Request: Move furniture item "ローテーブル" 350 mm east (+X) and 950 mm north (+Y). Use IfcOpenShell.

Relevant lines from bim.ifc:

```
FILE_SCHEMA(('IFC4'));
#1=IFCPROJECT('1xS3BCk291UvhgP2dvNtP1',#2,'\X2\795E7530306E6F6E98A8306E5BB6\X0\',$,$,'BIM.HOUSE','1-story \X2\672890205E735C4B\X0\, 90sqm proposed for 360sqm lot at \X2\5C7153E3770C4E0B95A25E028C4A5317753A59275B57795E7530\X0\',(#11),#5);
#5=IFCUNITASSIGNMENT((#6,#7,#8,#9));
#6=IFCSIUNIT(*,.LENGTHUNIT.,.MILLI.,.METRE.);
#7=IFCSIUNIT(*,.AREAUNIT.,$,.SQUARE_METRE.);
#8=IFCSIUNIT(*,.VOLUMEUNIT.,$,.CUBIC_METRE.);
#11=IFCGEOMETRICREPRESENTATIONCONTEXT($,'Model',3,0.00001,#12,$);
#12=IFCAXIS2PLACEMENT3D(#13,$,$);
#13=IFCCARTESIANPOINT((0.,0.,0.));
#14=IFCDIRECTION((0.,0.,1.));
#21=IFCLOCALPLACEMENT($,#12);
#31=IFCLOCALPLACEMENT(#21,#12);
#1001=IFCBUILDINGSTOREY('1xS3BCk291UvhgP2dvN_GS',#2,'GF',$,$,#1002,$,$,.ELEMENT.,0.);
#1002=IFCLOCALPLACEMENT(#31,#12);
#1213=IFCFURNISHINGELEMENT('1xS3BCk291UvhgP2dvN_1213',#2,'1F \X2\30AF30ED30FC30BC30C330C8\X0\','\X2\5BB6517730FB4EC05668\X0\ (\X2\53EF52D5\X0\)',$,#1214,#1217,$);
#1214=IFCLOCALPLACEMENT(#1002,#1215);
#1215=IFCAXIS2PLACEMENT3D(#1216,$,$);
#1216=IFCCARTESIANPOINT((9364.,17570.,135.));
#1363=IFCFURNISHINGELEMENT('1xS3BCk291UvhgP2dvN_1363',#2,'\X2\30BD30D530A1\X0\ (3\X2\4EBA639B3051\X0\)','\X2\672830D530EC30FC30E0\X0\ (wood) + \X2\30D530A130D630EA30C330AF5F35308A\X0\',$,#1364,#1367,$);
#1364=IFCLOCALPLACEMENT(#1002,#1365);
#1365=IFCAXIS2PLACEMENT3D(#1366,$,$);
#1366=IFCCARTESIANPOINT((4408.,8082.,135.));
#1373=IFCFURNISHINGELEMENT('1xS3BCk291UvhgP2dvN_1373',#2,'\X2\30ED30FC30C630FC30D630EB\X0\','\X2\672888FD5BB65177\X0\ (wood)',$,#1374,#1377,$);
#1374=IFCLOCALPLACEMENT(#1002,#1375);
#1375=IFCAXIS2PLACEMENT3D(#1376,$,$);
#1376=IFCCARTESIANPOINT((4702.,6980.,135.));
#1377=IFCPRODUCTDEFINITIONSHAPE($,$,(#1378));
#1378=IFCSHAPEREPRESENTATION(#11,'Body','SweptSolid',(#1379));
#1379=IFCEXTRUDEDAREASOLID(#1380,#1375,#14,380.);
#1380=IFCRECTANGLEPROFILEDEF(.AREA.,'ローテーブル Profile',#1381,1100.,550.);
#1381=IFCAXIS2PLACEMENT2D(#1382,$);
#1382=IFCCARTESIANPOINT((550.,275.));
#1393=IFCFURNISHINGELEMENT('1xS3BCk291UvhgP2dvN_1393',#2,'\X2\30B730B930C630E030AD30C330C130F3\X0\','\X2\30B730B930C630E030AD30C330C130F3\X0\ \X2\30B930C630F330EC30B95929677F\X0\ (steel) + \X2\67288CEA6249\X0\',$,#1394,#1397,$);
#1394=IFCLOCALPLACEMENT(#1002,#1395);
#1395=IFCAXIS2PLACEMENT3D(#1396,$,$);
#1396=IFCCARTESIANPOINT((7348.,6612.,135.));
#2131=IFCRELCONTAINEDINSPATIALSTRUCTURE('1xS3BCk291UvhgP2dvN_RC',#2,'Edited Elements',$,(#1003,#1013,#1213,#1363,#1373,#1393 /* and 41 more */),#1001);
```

```python
import ifcopenshell
import ifcopenshell.api.geometry
import ifcopenshell.util.placement
import ifcopenshell.util.unit

model = ifcopenshell.open("bim.ifc")
unit_scale = ifcopenshell.util.unit.calculate_unit_scale(model)

item = model.by_guid("1xS3BCk291UvhgP2dvN_1373")
matrix = ifcopenshell.util.placement.get_local_placement(item.ObjectPlacement)
matrix[0, 3] += 0.35 / unit_scale
matrix[1, 3] += 0.95 / unit_scale
ifcopenshell.api.geometry.edit_object_placement(model, product=item, matrix=matrix, is_si=False)

print(ifcopenshell.util.placement.get_local_placement(item.ObjectPlacement).round(3) + 0.0)

model.write("bim_rev.ifc")
```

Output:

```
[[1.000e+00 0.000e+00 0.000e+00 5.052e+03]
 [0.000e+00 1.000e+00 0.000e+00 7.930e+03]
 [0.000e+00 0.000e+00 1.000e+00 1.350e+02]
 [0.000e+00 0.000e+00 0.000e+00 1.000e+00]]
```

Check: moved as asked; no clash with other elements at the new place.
